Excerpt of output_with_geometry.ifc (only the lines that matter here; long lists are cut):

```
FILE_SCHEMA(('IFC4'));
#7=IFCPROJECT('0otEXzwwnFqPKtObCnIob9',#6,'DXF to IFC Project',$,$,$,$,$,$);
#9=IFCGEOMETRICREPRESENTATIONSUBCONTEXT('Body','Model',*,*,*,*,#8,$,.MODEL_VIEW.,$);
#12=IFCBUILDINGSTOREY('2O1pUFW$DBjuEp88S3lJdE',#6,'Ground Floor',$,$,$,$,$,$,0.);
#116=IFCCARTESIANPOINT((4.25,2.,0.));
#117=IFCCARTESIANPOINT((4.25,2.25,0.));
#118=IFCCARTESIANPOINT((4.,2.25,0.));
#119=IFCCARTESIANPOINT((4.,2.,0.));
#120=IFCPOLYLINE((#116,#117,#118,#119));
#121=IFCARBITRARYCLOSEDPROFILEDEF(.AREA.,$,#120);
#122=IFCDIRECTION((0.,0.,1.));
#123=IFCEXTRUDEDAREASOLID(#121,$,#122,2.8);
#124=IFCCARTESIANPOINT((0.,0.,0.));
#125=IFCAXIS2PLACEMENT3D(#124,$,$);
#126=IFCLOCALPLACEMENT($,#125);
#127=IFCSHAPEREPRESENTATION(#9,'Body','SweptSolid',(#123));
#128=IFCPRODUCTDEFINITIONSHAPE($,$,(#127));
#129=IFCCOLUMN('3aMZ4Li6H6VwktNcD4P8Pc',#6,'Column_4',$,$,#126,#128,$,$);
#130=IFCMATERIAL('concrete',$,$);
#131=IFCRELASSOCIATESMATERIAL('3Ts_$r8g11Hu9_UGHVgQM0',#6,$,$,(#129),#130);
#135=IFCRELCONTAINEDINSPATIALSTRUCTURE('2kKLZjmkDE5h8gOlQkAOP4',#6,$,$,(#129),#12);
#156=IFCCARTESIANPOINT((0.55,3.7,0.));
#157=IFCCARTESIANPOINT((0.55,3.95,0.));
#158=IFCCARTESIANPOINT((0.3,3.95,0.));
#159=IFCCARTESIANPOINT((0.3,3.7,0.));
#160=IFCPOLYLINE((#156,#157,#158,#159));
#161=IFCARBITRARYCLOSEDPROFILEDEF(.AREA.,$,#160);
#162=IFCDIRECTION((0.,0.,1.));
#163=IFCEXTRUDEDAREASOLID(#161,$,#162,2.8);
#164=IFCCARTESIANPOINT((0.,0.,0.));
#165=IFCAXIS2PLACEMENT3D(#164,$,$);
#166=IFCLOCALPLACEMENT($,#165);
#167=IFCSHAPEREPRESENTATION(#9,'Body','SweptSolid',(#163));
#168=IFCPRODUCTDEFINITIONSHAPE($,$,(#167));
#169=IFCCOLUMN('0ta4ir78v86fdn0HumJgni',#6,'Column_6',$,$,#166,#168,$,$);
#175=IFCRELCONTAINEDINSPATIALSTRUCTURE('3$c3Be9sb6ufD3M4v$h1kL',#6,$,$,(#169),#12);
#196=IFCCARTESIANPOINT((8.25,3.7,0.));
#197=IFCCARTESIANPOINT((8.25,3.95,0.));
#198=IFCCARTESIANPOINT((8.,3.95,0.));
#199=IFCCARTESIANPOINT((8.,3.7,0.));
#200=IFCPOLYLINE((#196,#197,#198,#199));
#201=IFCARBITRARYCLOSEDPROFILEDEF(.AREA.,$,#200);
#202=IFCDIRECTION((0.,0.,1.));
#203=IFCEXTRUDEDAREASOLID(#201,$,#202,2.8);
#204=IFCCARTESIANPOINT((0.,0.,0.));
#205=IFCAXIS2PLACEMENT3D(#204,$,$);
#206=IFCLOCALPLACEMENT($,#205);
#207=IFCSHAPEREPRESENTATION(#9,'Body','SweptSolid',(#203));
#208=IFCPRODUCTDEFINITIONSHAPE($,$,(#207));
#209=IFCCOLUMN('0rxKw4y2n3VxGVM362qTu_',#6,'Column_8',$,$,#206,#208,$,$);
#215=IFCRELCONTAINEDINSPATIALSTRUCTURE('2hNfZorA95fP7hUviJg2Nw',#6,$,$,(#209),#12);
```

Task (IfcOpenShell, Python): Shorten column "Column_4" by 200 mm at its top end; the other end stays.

```python
import ifcopenshell
import ifcopenshell.util.representation
import ifcopenshell.util.unit

model = ifcopenshell.open("output_with_geometry.ifc")
unit_scale = ifcopenshell.util.unit.calculate_unit_scale(model)

member = model.by_guid("3aMZ4Li6H6VwktNcD4P8Pc")
change = -0.2 / unit_scale

# The extrusion runs towards the end named, so only its depth changes.
body = ifcopenshell.util.representation.get_representation(member, "Model", "Body")
solid = body.Items[0]
old_length = solid.Depth
solid.Depth += change

print(f"length {old_length:g} -> {solid.Depth:g}")

model.write("output_with_geometry_v2.ifc")
```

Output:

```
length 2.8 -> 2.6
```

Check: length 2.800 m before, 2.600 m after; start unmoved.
